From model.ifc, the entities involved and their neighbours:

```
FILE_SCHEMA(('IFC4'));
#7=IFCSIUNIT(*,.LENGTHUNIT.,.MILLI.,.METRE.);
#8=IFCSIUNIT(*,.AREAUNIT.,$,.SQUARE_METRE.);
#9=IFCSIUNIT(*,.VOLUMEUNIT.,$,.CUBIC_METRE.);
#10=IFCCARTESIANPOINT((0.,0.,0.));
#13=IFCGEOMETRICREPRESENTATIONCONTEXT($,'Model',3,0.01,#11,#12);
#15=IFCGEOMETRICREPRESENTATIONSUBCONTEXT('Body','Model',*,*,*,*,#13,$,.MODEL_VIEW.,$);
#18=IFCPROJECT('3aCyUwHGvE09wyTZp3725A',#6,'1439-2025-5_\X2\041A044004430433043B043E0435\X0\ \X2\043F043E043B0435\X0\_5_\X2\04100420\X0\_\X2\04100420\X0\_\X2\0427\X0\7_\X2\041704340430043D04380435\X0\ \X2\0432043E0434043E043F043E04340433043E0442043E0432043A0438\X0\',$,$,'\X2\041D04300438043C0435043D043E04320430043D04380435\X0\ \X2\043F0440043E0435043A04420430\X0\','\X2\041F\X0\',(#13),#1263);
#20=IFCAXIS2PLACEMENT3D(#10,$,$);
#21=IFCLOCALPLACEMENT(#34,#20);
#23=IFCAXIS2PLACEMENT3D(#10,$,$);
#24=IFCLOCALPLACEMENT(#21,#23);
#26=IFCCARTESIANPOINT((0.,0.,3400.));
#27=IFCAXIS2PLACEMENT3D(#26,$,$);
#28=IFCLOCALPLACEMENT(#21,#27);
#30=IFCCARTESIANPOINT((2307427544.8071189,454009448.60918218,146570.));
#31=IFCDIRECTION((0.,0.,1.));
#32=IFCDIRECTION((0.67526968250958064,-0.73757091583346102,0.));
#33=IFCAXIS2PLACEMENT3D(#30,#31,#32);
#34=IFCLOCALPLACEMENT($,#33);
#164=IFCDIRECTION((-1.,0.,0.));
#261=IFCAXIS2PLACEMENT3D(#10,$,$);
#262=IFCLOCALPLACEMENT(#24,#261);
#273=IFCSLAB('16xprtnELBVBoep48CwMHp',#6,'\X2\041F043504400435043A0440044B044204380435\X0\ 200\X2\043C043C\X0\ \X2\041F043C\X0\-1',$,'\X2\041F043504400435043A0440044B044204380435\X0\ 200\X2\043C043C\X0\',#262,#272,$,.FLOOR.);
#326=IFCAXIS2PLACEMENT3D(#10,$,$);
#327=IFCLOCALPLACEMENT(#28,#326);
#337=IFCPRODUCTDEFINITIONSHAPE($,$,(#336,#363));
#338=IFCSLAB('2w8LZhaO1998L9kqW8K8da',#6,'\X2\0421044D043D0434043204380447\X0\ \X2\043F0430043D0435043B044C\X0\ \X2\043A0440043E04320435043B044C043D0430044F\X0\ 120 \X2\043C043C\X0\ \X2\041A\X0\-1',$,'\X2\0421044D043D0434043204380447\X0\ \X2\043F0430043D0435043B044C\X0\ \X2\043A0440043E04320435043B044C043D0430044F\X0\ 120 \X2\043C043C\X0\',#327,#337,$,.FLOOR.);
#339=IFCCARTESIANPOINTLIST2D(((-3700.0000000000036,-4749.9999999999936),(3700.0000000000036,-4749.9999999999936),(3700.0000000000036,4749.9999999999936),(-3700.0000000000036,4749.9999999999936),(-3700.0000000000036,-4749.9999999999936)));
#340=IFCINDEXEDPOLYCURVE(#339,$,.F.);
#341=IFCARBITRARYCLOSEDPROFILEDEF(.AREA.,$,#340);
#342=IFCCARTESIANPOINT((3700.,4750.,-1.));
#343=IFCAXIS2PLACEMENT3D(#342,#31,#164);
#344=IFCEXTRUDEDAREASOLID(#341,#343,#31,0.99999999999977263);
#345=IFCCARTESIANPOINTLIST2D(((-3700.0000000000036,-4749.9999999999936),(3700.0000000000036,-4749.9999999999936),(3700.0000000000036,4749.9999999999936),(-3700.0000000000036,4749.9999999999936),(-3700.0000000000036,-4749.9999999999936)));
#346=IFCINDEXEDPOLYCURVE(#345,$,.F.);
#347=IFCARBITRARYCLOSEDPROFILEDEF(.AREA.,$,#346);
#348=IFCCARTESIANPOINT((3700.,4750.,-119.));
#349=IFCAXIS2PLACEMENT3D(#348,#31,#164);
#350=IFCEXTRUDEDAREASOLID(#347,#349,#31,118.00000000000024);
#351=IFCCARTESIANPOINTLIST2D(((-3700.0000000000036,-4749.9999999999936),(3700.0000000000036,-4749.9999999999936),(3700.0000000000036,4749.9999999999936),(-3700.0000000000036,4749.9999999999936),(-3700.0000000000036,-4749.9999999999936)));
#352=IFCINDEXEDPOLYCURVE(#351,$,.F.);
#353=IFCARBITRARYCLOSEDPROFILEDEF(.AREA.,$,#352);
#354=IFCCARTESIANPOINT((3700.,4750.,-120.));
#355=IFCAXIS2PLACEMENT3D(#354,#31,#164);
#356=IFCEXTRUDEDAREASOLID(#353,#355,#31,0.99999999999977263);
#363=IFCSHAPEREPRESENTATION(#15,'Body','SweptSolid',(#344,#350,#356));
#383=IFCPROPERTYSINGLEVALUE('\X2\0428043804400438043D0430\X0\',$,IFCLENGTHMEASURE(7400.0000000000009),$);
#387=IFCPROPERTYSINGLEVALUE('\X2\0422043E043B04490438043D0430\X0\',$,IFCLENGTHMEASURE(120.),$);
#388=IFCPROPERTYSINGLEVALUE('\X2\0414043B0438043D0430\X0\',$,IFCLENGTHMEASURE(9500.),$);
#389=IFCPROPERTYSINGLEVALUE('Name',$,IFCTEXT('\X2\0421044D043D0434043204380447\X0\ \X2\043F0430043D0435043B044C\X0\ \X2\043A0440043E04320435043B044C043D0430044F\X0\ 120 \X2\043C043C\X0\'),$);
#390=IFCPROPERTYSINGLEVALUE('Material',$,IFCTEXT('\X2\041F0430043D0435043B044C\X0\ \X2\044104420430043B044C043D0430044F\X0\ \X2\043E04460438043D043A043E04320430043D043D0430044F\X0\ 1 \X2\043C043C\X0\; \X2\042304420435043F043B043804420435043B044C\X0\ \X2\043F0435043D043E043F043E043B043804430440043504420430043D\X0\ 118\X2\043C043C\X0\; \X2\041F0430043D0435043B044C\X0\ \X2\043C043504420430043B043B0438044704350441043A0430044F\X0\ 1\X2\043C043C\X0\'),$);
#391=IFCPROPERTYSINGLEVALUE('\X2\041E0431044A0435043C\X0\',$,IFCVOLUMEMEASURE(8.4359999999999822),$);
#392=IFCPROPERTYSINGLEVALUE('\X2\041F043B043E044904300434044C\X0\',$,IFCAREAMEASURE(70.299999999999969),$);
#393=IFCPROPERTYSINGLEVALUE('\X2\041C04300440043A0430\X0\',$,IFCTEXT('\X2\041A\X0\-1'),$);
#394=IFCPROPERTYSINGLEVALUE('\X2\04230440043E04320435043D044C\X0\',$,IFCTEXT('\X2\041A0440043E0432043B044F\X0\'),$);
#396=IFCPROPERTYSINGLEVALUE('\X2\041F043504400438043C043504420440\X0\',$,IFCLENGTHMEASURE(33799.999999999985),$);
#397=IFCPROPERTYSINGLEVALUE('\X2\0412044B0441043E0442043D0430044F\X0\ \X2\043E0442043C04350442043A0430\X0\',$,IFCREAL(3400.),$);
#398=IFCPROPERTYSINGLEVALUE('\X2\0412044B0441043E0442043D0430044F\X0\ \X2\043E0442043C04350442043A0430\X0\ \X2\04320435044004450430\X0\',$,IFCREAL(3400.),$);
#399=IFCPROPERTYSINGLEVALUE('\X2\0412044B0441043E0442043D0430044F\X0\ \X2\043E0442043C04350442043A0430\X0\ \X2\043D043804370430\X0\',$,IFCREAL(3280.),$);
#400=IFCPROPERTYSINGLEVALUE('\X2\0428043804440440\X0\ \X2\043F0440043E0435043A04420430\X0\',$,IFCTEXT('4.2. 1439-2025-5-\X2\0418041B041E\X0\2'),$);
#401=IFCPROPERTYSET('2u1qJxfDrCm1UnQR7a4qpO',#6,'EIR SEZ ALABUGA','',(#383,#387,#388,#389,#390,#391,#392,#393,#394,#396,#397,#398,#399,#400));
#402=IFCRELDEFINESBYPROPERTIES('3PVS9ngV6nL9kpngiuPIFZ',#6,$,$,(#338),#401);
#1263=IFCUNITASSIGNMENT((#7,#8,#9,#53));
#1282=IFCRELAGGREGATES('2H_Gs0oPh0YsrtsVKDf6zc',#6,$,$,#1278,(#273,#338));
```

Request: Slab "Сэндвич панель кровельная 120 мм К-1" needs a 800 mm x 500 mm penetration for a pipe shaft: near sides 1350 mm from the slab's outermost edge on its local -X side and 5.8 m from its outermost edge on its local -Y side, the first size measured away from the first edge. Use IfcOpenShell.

```python
import numpy as np
import ifcopenshell
import ifcopenshell.api.feature
import ifcopenshell.api.geometry
import ifcopenshell.api.pset
import ifcopenshell.api.root
import ifcopenshell.geom
import ifcopenshell.util.element
import ifcopenshell.util.placement
import ifcopenshell.util.representation
import ifcopenshell.util.shape
import ifcopenshell.util.unit

model = ifcopenshell.open("model.ifc")
unit_scale = ifcopenshell.util.unit.calculate_unit_scale(model)
area_scale = ifcopenshell.util.unit.calculate_unit_scale(model, "AREAUNIT")
volume_scale = ifcopenshell.util.unit.calculate_unit_scale(model, "VOLUMEUNIT")
settings = ifcopenshell.geom.settings()


def volume(element):
    """Net volume in cubic metres, openings subtracted."""
    shape = ifcopenshell.geom.create_shape(settings, element)
    return ifcopenshell.util.shape.get_volume(shape.geometry)


slab = model.by_id(338)
before = volume(slab)

# Extent in the slab's own axes, in metres. The edges named are its -X and -Y sides.
slab_shape = ifcopenshell.geom.create_shape(settings, slab)
vertices = ifcopenshell.util.shape.get_vertices(slab_shape.geometry)
x_min, y_min, bottom = vertices.min(axis=0)
top = vertices[:, 2].max()

opening = ifcopenshell.api.root.create_entity(model, ifc_class="IfcOpeningElement", name="Pipe shaft opening", predefined_type="OPENING")
context = ifcopenshell.util.representation.get_context(model, "Model", "Body", "MODEL_VIEW")
width, depth = 0.8, 0.5
outline = [(0.0, 0.0), (width, 0.0), (width, depth), (0.0, depth), (0.0, 0.0)]
# Overshoot both faces by 50 mm so the cut is clean.
shape = ifcopenshell.api.geometry.add_slab_representation(
    model, context=context, depth=top - bottom + 0.1, polyline=outline
)
ifcopenshell.api.geometry.assign_representation(model, product=opening, representation=shape)

matrix = ifcopenshell.util.placement.get_local_placement(slab.ObjectPlacement)
matrix[:, 3] = matrix @ np.append(np.array([x_min + 1.35, y_min + 5.8, bottom - 0.05]) / unit_scale, 1.0)
ifcopenshell.api.geometry.edit_object_placement(model, product=opening, matrix=matrix, is_si=False)
ifcopenshell.api.feature.add_feature(model, feature=opening, element=slab)

after = volume(slab)

# Update the slab's stored quantities.
pset = model.by_id(ifcopenshell.util.element.get_pset(slab, "EIR SEZ ALABUGA", should_inherit=False)["id"])
ifcopenshell.api.pset.edit_pset(model, pset=pset, properties={
    "Объем": model.create_entity("IfcVolumeMeasure", after / volume_scale),
    "Площадь": model.create_entity("IfcAreaMeasure", after / (top - bottom) / area_scale),
})

print(f"slab volume {before:.3f} -> {after:.3f} m3")

model.write("model_v2.ifc")
```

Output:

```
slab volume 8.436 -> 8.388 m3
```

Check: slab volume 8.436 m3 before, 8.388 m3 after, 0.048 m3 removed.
